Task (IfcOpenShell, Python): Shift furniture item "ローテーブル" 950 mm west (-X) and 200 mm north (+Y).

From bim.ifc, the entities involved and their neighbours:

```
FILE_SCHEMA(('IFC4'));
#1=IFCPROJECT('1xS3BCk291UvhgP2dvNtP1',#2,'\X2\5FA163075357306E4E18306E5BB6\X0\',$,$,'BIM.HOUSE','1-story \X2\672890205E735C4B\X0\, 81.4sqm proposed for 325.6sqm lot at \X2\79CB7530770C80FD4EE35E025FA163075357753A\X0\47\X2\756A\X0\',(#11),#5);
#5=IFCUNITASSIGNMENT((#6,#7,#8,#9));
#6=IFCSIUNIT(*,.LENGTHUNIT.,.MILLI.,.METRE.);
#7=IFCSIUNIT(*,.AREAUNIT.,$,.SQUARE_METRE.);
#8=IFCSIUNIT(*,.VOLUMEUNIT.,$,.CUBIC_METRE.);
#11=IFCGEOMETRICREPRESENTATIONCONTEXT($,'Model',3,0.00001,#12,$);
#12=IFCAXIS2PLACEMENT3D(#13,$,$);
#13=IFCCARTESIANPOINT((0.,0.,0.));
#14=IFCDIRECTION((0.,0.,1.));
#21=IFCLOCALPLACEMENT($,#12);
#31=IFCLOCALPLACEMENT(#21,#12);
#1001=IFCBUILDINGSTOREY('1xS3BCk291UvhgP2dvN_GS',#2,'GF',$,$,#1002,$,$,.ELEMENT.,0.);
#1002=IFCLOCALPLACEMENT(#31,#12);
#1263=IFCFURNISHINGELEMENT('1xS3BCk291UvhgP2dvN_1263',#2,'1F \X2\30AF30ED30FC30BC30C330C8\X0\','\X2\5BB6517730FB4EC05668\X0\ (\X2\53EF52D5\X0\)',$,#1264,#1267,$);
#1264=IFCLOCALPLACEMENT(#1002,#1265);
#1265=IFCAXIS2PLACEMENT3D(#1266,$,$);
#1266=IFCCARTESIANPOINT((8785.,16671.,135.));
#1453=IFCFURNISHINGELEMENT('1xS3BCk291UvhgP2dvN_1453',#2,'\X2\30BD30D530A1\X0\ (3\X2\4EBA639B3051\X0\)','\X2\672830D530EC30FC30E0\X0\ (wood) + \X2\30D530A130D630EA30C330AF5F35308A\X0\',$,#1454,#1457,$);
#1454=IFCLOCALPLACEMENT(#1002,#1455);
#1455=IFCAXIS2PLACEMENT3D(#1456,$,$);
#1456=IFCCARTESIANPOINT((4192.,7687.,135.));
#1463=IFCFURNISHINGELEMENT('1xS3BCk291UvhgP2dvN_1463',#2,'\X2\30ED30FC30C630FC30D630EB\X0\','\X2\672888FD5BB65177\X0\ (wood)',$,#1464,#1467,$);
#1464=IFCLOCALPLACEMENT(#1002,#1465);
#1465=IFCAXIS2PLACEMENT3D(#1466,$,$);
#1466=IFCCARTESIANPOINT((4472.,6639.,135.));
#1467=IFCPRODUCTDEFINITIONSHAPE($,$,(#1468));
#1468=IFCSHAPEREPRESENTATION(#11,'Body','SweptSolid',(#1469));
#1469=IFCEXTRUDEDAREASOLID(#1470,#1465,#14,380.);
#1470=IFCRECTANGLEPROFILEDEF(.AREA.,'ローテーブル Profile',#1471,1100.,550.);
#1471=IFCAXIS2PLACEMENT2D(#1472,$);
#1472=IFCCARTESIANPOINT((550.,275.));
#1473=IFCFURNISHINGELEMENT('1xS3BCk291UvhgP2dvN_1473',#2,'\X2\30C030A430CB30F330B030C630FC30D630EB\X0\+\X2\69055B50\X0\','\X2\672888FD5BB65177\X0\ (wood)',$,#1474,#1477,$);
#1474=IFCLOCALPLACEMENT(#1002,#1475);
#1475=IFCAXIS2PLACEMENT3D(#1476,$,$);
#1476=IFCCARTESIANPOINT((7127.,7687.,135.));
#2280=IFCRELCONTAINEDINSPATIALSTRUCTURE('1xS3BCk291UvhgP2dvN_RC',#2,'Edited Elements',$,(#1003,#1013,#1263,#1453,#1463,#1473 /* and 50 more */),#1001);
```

```python
import ifcopenshell
import ifcopenshell.api.geometry
import ifcopenshell.util.placement

model = ifcopenshell.open("bim.ifc")

item = model.by_guid("1xS3BCk291UvhgP2dvN_1463")
matrix = ifcopenshell.util.placement.get_local_placement(item.ObjectPlacement)
matrix[0, 3] -= 950.0
matrix[1, 3] += 200.0
ifcopenshell.api.geometry.edit_object_placement(model, product=item, matrix=matrix, is_si=False)

print(ifcopenshell.util.placement.get_local_placement(item.ObjectPlacement).round(3) + 0.0)

model.write("bim_rev.ifc")
```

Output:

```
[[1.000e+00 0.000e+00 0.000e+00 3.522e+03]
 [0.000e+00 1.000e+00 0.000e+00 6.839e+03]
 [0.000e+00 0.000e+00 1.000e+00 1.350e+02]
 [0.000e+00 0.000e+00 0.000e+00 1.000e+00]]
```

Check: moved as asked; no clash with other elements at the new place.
